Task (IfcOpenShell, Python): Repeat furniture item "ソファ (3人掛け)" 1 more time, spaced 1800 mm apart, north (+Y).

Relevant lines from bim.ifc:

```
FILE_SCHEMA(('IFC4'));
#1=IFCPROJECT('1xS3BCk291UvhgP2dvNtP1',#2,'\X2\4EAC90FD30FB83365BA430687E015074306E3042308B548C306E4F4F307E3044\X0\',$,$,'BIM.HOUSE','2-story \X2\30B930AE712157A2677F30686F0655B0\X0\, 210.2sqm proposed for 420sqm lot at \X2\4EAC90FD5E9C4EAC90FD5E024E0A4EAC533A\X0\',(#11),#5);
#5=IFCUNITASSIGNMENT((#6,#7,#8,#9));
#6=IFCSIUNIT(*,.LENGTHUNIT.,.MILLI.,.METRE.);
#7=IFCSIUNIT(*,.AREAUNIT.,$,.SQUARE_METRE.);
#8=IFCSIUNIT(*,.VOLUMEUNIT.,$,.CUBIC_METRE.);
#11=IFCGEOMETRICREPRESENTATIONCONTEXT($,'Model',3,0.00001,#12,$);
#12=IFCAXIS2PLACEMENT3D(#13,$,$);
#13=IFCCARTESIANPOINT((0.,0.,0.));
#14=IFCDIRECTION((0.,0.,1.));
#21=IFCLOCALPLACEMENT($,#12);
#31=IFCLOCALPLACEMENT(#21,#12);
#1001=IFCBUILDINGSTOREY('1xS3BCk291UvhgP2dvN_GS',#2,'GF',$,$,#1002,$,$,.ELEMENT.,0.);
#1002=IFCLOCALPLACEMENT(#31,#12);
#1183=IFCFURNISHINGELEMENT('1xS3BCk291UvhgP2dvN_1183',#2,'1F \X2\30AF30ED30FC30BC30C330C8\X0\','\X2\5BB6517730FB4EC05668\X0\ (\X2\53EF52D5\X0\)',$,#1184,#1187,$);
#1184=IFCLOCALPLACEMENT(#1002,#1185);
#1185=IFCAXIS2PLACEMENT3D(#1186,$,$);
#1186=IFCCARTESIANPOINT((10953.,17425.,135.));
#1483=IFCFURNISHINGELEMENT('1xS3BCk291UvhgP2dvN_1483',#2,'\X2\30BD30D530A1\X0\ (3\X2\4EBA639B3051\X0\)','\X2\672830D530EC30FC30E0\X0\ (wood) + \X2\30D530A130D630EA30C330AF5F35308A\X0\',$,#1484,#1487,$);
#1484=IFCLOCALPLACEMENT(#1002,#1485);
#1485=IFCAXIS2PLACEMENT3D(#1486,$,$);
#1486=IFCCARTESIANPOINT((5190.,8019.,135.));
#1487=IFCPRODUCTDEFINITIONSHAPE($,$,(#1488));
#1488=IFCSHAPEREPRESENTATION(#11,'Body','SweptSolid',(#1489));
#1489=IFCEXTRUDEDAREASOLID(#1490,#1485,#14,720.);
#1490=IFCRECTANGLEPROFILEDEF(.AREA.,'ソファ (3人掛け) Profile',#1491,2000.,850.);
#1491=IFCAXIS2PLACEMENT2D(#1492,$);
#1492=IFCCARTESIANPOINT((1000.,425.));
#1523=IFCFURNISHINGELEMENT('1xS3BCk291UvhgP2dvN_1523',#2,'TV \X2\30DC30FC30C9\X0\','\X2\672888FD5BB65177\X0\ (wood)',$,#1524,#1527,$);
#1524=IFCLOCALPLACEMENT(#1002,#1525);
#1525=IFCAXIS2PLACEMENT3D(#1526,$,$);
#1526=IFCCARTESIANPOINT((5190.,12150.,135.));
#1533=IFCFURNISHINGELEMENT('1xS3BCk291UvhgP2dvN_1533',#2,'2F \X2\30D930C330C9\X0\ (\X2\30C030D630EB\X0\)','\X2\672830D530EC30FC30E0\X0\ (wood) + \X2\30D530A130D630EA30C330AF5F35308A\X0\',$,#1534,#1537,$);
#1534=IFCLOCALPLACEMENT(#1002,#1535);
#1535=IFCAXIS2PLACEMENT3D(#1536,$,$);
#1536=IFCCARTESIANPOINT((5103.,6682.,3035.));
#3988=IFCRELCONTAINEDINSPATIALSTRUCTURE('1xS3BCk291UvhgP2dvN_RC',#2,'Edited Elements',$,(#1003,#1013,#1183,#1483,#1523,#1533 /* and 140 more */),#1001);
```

```python
import numpy as np
import ifcopenshell
import ifcopenshell.api.geometry
import ifcopenshell.api.root
import ifcopenshell.util.element
import ifcopenshell.util.placement
import ifcopenshell.util.unit

model = ifcopenshell.open("bim.ifc")
unit_scale = ifcopenshell.util.unit.calculate_unit_scale(model)


def reuse_history(source, copy):
    """copy_class also copies each property set's owner history, people and application; keep the originals."""
    for rel in copy.IsDefinedBy:
        if rel.is_a("IfcRelDefinesByProperties") and (history := rel.RelatingPropertyDefinition.OwnerHistory):
            rel.RelatingPropertyDefinition.OwnerHistory = source.OwnerHistory
            ifcopenshell.util.element.remove_deep2(model, history)


source = model.by_id(1483)
base = ifcopenshell.util.placement.get_local_placement(source.ObjectPlacement)
step = np.array([0.0, 1.0, 0.0]) * 1.8 / unit_scale

for i in range(1, 2):
    copy = ifcopenshell.api.root.copy_class(model, product=source)
    copy.Representation = ifcopenshell.util.element.copy_deep(
        model, source.Representation, exclude=["IfcGeometricRepresentationContext", "IfcRepresentationMap"]
    )
    reuse_history(source, copy)
    matrix = base.copy()
    matrix[:3, 3] += i * step
    print("added at", matrix[:3, 3].round(3) + 0.0)
    ifcopenshell.api.geometry.edit_object_placement(model, product=copy, matrix=matrix, is_si=False)

model.write("bim-out.ifc")
```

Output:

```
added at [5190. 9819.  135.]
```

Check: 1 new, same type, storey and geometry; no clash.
